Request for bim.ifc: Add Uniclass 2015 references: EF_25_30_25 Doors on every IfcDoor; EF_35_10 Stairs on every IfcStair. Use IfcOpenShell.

First a look at what the model holds.

```python
import ifcopenshell

model = ifcopenshell.open("bim.ifc")
print(model.schema)
print("classifications:", [c.Name for c in model.by_type("IfcClassification")])
for ifc_class in ("IfcDoor", "IfcRoof", "IfcStair", "IfcWall", "IfcWindow"):
    print(ifc_class, len(model.by_type(ifc_class)))
```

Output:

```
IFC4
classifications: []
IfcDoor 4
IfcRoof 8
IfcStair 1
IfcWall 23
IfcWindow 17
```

```python
import ifcopenshell
import ifcopenshell.api.classification

model = ifcopenshell.open("bim.ifc")

system = ifcopenshell.api.classification.add_classification(model, classification="Uniclass 2015")

codes = {
    "IfcDoor": ("EF_25_30_25", "Doors"),
    "IfcStair": ("EF_35_10", "Stairs"),
}
for ifc_class, (code, name) in codes.items():
    products = model.by_type(ifc_class)
    ifcopenshell.api.classification.add_reference(
        model, products=products, classification=system, identification=code, name=name
    )
    print(code, len(products))

model.write("bim_edited.ifc")
```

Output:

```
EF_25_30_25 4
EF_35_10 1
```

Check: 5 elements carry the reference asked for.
